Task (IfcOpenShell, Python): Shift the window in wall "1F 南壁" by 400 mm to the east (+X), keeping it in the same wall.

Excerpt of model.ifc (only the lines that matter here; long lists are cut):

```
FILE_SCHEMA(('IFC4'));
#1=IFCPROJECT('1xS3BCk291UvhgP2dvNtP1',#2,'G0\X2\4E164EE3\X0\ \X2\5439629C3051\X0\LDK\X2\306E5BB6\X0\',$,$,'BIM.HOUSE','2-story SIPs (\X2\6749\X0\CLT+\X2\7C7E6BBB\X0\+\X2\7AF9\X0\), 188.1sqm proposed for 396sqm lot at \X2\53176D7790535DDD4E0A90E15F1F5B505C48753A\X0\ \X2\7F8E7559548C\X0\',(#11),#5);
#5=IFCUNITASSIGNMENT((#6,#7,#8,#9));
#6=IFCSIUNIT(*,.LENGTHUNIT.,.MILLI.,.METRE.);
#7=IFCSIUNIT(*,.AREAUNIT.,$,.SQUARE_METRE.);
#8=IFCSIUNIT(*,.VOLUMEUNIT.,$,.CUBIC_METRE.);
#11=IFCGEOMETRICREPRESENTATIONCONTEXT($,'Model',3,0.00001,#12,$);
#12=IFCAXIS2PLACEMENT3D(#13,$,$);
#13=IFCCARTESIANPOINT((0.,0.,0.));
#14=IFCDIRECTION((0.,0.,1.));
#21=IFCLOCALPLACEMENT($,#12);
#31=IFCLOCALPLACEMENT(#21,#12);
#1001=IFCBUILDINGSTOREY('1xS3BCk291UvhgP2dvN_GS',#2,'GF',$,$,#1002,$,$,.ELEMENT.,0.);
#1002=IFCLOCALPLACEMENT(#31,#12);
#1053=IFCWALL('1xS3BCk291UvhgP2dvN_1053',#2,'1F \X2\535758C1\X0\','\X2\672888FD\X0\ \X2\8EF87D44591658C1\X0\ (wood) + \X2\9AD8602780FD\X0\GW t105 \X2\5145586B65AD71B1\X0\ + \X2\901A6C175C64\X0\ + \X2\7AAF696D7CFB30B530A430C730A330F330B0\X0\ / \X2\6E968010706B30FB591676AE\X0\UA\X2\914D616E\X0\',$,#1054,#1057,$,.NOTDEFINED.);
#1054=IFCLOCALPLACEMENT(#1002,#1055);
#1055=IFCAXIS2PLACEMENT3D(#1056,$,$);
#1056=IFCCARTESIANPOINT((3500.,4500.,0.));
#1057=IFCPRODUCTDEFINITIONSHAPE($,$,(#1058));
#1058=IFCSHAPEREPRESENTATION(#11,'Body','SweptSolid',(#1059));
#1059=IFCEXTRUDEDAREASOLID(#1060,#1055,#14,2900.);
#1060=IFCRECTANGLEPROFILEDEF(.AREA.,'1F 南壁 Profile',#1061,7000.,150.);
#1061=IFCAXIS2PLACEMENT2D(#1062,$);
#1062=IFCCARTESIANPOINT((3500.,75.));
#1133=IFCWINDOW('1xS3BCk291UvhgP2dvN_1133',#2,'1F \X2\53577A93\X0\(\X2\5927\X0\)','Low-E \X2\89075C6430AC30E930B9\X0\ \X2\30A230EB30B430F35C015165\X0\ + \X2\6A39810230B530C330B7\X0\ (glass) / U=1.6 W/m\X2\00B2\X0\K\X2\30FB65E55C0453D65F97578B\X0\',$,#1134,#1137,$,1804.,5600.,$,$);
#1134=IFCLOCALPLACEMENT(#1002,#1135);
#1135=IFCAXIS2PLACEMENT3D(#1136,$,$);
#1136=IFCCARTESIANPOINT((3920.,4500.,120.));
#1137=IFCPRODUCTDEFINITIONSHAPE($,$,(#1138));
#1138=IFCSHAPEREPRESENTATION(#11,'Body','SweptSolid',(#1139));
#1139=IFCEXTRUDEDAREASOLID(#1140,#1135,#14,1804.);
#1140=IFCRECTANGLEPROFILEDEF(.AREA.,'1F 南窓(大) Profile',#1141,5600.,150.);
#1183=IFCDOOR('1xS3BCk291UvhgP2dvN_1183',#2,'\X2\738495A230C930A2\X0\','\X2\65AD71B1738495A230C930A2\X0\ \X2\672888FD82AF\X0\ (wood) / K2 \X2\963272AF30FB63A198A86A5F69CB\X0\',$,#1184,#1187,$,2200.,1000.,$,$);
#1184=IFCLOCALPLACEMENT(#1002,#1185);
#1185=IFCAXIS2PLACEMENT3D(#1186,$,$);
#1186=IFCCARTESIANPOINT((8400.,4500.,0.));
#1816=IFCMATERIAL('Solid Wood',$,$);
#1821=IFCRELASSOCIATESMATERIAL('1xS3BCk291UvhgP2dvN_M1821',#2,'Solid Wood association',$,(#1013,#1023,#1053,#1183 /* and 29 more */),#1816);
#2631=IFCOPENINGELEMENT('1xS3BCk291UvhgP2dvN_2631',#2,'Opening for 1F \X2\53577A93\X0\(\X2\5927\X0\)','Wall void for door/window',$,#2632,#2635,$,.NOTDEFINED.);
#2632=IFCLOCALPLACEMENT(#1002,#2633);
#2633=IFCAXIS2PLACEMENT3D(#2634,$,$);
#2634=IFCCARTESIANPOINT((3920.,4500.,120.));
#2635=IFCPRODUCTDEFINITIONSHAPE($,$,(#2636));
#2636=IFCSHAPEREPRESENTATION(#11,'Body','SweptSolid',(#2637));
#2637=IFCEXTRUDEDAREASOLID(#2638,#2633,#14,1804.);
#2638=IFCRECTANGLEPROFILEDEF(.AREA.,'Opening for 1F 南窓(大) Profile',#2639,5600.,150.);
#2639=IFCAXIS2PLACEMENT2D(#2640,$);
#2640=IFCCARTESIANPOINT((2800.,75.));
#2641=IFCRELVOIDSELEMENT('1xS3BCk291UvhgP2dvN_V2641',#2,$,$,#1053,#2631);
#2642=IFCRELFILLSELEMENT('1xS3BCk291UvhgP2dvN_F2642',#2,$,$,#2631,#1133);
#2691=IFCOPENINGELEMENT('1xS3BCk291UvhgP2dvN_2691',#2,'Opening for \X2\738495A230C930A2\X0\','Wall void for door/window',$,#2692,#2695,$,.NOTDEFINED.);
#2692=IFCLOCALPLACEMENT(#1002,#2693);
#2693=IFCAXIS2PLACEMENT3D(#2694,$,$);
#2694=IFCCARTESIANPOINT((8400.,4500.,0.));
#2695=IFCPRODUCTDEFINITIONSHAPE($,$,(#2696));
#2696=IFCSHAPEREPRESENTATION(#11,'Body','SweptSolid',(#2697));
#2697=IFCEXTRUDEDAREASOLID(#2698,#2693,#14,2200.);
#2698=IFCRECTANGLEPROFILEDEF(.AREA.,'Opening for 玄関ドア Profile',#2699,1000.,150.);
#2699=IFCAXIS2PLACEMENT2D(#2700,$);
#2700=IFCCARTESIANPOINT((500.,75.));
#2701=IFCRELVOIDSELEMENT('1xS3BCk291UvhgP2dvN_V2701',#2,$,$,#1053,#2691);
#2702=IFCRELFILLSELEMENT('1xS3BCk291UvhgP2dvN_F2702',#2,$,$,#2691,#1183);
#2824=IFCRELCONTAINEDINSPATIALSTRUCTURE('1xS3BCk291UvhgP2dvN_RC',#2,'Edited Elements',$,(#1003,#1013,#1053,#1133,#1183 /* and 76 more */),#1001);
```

```python
import ifcopenshell
import ifcopenshell.api.geometry
import ifcopenshell.util.placement

model = ifcopenshell.open("model.ifc")

window = model.by_guid("1xS3BCk291UvhgP2dvN_1133")
opening = window.FillsVoids[0].RelatingOpeningElement
wall = opening.VoidsElements[0].RelatingBuildingElement

wall_matrix = ifcopenshell.util.placement.get_local_placement(wall.ObjectPlacement)
shift = wall_matrix[:3, 0] * 400.0
before = ifcopenshell.util.placement.get_local_placement(window.ObjectPlacement)[:3, 3].copy()

# The window is not placed relative to its opening, so move both.
for product in (opening, window):
    matrix = ifcopenshell.util.placement.get_local_placement(product.ObjectPlacement)
    matrix[:3, 3] += shift
    ifcopenshell.api.geometry.edit_object_placement(model, product=product, matrix=matrix, is_si=False)

after = ifcopenshell.util.placement.get_local_placement(window.ObjectPlacement)[:3, 3]
print("window moved by", (after - before).round(3) + 0.0)

model.write("model_edited.ifc")
```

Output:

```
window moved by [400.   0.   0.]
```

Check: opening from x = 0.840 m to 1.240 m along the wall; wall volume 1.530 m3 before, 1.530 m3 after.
